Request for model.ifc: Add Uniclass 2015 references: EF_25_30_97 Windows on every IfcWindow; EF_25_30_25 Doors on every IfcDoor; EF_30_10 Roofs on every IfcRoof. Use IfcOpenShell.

First a look at what the model holds.

```python
import ifcopenshell

model = ifcopenshell.open("model.ifc")
print(model.schema)
print("classifications:", [c.Name for c in model.by_type("IfcClassification")])
for ifc_class in ("IfcDoor", "IfcRoof", "IfcStair", "IfcWall", "IfcWindow"):
    print(ifc_class, len(model.by_type(ifc_class)))
```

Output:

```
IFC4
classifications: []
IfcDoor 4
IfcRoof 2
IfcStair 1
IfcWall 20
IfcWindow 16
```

```python
import ifcopenshell
import ifcopenshell.api.classification

model = ifcopenshell.open("model.ifc")

system = ifcopenshell.api.classification.add_classification(model, classification="Uniclass 2015")

codes = {
    "IfcWindow": ("EF_25_30_97", "Windows"),
    "IfcDoor": ("EF_25_30_25", "Doors"),
    "IfcRoof": ("EF_30_10", "Roofs"),
}
for ifc_class, (code, name) in codes.items():
    products = model.by_type(ifc_class)
    ifcopenshell.api.classification.add_reference(
        model, products=products, classification=system, identification=code, name=name
    )
    print(code, len(products))

model.write("model_rev.ifc")
```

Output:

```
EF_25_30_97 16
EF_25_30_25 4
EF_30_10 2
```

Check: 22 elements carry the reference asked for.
